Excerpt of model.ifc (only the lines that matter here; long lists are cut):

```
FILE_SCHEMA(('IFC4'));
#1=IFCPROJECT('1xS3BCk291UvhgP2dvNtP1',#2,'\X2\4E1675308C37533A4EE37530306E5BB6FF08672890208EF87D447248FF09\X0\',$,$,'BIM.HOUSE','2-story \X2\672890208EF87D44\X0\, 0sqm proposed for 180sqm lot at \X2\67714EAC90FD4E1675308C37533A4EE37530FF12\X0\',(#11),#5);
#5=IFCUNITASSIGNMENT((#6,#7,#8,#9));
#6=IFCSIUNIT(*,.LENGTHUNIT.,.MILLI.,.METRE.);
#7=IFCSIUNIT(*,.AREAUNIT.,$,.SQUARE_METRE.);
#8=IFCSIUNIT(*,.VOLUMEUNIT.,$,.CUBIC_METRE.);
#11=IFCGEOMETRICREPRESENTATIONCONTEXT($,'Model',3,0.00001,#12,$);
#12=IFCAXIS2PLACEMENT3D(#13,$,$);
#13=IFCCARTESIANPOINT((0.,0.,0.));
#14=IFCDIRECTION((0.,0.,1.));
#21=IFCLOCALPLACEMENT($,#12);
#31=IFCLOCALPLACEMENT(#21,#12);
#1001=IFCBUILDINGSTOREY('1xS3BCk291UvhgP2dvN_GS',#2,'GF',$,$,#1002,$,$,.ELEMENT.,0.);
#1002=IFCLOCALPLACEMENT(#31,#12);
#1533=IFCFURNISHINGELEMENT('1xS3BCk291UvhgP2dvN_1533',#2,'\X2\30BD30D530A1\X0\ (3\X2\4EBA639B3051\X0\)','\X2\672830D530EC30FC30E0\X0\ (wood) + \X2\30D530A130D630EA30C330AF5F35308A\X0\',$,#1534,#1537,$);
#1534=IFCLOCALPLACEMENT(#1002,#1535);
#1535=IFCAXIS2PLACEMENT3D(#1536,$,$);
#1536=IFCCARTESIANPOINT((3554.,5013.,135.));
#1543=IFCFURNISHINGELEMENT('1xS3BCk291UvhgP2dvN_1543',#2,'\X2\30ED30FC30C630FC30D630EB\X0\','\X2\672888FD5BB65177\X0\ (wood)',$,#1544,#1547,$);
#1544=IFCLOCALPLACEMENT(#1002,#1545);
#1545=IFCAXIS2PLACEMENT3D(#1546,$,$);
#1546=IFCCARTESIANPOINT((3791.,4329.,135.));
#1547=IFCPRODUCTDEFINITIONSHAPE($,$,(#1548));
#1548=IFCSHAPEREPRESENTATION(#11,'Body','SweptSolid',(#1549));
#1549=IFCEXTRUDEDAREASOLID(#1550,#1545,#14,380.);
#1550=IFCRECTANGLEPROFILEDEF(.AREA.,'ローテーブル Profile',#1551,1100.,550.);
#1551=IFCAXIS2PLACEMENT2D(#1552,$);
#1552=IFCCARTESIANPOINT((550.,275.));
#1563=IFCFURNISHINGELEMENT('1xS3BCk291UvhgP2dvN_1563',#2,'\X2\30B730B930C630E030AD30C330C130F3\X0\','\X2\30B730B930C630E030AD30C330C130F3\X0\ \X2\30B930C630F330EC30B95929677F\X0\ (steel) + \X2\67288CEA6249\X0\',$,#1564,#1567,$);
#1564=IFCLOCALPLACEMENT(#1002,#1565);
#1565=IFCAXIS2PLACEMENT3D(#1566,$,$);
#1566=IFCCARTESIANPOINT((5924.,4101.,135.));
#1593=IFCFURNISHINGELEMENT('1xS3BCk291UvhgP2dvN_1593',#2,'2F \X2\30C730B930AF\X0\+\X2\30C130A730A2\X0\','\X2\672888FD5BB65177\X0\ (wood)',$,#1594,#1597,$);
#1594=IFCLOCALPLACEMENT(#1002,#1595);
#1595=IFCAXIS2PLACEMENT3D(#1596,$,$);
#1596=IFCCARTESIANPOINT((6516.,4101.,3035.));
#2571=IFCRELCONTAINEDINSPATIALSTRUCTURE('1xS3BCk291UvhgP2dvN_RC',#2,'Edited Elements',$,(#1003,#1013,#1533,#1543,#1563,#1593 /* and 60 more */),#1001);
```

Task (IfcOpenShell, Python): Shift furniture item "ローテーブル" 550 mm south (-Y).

```python
import ifcopenshell
import ifcopenshell.api.geometry
import ifcopenshell.util.placement

model = ifcopenshell.open("model.ifc")

item = model.by_guid("1xS3BCk291UvhgP2dvN_1543")
matrix = ifcopenshell.util.placement.get_local_placement(item.ObjectPlacement)
matrix[1, 3] -= 550.0
ifcopenshell.api.geometry.edit_object_placement(model, product=item, matrix=matrix, is_si=False)

print(ifcopenshell.util.placement.get_local_placement(item.ObjectPlacement).round(3) + 0.0)

model.write("model_rev.ifc")
```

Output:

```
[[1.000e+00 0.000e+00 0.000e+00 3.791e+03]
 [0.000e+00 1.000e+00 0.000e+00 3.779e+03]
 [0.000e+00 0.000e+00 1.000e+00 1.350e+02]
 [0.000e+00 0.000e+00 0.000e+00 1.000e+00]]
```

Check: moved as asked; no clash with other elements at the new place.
